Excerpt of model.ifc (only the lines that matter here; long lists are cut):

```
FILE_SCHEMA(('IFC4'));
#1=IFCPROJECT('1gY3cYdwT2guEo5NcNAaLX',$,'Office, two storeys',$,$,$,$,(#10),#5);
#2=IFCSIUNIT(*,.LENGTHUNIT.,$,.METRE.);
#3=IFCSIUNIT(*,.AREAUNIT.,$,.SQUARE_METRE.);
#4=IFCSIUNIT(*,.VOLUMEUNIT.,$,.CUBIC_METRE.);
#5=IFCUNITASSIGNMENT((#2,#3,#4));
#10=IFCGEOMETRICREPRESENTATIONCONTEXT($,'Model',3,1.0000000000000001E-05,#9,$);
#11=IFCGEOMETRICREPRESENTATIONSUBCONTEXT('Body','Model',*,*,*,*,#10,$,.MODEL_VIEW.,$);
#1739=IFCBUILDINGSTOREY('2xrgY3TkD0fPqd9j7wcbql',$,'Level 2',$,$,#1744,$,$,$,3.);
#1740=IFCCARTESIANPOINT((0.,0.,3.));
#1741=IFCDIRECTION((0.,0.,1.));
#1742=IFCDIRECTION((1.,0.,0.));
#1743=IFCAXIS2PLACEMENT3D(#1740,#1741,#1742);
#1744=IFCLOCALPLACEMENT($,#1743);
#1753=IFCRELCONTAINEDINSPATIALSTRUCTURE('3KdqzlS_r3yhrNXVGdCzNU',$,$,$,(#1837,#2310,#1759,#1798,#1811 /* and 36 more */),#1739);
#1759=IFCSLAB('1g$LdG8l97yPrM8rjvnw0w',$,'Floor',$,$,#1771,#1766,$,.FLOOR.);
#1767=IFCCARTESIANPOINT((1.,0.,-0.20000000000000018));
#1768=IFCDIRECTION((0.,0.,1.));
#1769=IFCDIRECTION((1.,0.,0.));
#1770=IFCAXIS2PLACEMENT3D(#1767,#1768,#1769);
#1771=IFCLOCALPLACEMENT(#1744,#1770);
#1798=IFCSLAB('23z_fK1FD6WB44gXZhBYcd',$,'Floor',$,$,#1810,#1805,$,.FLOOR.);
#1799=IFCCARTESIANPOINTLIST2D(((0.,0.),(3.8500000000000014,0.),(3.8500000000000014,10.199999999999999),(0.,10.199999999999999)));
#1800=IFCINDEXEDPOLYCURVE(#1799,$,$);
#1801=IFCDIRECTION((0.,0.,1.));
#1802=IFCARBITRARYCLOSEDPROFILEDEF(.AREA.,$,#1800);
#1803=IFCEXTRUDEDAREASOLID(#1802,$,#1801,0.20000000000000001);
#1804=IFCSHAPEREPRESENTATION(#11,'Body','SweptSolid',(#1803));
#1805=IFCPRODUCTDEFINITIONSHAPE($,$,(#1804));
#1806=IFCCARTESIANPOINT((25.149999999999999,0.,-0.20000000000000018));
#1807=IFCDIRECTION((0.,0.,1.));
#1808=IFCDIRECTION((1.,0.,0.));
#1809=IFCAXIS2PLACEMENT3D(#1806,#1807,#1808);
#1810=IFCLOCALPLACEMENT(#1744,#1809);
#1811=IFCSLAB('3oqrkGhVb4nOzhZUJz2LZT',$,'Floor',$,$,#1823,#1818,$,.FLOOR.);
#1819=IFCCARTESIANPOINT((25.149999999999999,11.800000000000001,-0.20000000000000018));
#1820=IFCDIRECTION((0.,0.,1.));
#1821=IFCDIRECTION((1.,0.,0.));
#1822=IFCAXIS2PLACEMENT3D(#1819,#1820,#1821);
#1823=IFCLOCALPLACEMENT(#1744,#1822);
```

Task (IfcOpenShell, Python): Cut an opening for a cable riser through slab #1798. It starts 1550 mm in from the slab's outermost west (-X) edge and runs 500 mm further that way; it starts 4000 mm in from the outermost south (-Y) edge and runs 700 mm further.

```python
import numpy as np
import ifcopenshell
import ifcopenshell.api.feature
import ifcopenshell.api.geometry
import ifcopenshell.api.root
import ifcopenshell.geom
import ifcopenshell.util.placement
import ifcopenshell.util.representation
import ifcopenshell.util.shape
import ifcopenshell.util.unit

model = ifcopenshell.open("model.ifc")
unit_scale = ifcopenshell.util.unit.calculate_unit_scale(model)
settings = ifcopenshell.geom.settings()


def volume(element):
    """Net volume in cubic metres, openings subtracted."""
    shape = ifcopenshell.geom.create_shape(settings, element)
    return ifcopenshell.util.shape.get_volume(shape.geometry)


slab = model.by_id(1798)
before = volume(slab)

# Extent in the slab's own axes, in metres. The edges named are its -X and -Y sides.
slab_shape = ifcopenshell.geom.create_shape(settings, slab)
vertices = ifcopenshell.util.shape.get_vertices(slab_shape.geometry)
x_min, y_min, bottom = vertices.min(axis=0)
top = vertices[:, 2].max()

opening = ifcopenshell.api.root.create_entity(model, ifc_class="IfcOpeningElement", name="Cable riser opening", predefined_type="OPENING")
context = ifcopenshell.util.representation.get_context(model, "Model", "Body", "MODEL_VIEW")
width, depth = 0.5, 0.7
outline = [(0.0, 0.0), (width, 0.0), (width, depth), (0.0, depth), (0.0, 0.0)]
# Overshoot both faces by 50 mm so the cut is clean.
shape = ifcopenshell.api.geometry.add_slab_representation(
    model, context=context, depth=top - bottom + 0.1, polyline=outline
)
ifcopenshell.api.geometry.assign_representation(model, product=opening, representation=shape)

matrix = ifcopenshell.util.placement.get_local_placement(slab.ObjectPlacement)
matrix[:, 3] = matrix @ np.append(np.array([x_min + 1.55, y_min + 4, bottom - 0.05]) / unit_scale, 1.0)
ifcopenshell.api.geometry.edit_object_placement(model, product=opening, matrix=matrix, is_si=False)
ifcopenshell.api.feature.add_feature(model, feature=opening, element=slab)

after = volume(slab)

print(f"slab volume {before:.3f} -> {after:.3f} m3")

model.write("model_rev.ifc")
```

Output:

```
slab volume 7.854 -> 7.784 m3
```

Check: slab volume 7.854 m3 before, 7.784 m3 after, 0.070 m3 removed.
